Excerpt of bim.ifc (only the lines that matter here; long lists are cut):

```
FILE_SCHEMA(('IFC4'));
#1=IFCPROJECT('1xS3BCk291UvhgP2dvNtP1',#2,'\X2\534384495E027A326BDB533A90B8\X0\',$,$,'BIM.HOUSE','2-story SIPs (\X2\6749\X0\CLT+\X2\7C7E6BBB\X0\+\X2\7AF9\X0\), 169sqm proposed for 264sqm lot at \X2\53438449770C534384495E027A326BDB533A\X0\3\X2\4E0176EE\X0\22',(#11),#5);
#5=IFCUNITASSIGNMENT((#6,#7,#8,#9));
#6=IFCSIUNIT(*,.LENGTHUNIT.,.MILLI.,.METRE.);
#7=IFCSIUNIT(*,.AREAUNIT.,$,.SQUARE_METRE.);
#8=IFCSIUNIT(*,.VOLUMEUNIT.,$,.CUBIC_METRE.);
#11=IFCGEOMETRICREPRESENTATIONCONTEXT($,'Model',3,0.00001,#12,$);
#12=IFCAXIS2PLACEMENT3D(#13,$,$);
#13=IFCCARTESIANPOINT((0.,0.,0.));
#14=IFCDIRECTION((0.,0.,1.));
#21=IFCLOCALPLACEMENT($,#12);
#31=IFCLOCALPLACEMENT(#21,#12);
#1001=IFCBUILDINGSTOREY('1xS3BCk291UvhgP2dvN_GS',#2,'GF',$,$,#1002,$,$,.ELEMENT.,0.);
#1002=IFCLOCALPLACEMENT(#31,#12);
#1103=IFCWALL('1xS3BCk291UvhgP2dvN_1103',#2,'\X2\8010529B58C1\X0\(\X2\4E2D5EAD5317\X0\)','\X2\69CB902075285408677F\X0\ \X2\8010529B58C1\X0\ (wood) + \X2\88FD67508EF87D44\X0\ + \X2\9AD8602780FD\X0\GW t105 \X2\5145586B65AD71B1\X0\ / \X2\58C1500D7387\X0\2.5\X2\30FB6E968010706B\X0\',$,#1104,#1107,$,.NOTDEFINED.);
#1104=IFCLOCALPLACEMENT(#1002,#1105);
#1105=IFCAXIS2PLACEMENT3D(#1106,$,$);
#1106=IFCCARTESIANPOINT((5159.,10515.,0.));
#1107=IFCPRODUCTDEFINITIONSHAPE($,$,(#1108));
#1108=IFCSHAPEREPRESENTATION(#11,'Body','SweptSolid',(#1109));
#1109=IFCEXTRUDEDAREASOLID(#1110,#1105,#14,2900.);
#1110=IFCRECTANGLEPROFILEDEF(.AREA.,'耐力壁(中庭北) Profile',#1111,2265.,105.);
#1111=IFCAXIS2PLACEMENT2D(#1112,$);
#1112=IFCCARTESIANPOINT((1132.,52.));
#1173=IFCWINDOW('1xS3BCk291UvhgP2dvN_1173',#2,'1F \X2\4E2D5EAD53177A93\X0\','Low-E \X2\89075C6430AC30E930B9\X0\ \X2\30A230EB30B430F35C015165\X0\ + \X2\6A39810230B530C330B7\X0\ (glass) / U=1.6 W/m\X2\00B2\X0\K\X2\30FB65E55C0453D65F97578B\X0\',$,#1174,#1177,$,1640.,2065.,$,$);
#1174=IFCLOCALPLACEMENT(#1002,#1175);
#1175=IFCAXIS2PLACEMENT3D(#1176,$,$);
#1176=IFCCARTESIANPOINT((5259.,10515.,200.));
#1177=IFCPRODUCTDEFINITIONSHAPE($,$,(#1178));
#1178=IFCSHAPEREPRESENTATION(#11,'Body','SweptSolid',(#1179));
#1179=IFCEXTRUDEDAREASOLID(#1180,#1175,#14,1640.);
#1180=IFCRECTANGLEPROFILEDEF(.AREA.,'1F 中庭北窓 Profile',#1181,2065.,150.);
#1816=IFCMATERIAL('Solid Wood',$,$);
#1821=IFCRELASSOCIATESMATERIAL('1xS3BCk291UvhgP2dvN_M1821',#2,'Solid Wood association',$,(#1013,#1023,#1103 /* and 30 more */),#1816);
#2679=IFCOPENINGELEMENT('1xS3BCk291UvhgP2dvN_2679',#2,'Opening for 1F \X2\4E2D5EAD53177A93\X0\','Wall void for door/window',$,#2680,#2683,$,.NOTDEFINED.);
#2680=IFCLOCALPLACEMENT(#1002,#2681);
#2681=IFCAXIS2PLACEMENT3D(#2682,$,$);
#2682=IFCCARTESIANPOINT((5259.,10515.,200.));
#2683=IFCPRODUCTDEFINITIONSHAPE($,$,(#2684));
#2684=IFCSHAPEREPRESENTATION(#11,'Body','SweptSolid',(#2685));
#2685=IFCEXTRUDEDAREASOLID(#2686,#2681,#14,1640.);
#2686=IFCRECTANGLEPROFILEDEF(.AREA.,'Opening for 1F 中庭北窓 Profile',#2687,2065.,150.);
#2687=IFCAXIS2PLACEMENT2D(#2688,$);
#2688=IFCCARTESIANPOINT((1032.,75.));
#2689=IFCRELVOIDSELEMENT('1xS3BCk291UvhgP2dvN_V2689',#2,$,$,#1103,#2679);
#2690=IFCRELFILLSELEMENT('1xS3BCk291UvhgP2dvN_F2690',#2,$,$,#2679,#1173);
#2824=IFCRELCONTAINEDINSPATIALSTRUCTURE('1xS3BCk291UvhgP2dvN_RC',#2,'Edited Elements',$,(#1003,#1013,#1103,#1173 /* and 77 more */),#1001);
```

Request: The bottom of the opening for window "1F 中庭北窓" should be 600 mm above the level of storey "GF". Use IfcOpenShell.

```python
import numpy as np
import ifcopenshell
import ifcopenshell.api.geometry
import ifcopenshell.geom
import ifcopenshell.util.element
import ifcopenshell.util.placement
import ifcopenshell.util.shape
import ifcopenshell.util.unit

model = ifcopenshell.open("bim.ifc")
unit_scale = ifcopenshell.util.unit.calculate_unit_scale(model)

window = model.by_id(1173)
opening = window.FillsVoids[0].RelatingOpeningElement
storey = ifcopenshell.util.element.get_container(window, ifc_class="IfcBuildingStorey")
level = ifcopenshell.util.placement.get_local_placement(storey.ObjectPlacement)[2, 3]

# The opening's origin need not be at the sill, so measure its lowest point.
shape = ifcopenshell.geom.create_shape(ifcopenshell.geom.settings(), opening)
bottom = ifcopenshell.util.shape.get_shape_bottom_elevation(shape, shape.geometry) / unit_scale
dz = level + 600.0 - bottom

shift = np.array([0.0, 0.0, dz])
# The window is not placed relative to its opening, so move both.
for product in (opening, window):
    matrix = ifcopenshell.util.placement.get_local_placement(product.ObjectPlacement)
    matrix[:3, 3] += shift
    ifcopenshell.api.geometry.edit_object_placement(model, product=product, matrix=matrix, is_si=False)

print(f"moved by {dz * unit_scale:+.3f} m")

model.write("bim_rev.ifc")
```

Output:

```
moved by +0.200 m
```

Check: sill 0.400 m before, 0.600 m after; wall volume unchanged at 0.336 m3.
